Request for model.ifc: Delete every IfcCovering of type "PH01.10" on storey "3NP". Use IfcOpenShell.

First a look at what the model holds.

```python
import ifcopenshell
import ifcopenshell.util.element

model = ifcopenshell.open("model.ifc")
print(model.schema)
storey = next(s for s in model.by_type("IfcBuildingStorey") if s.Name == "3NP")
coverings = [e for e in ifcopenshell.util.element.get_decomposition(storey) if e.is_a("IfcCovering")]
seen = {}
for e in coverings:
    element_type = ifcopenshell.util.element.get_type(e)
    name = element_type.Name if element_type not in (None, e) else None
    seen[name] = seen.get(name, 0) + 1
for name, count in sorted(seen.items(), key=str):
    print(count, "x", name)
```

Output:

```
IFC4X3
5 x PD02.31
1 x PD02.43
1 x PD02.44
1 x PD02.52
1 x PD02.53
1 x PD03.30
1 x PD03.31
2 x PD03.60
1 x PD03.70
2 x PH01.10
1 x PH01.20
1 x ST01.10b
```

```python
import ifcopenshell
import ifcopenshell.api.root
import ifcopenshell.util.element

model = ifcopenshell.open("model.ifc")

storey = next(s for s in model.by_type("IfcBuildingStorey") if s.Name == "3NP")
coverings = [e for e in ifcopenshell.util.element.get_decomposition(storey) if e.is_a("IfcCovering")]
targets = [e for e in coverings if (t := ifcopenshell.util.element.get_type(e)) not in (None, e) and t.Name == "PH01.10"]

for e in targets:
    ifcopenshell.api.root.remove_product(model, product=e)
print(len(targets), "removed")

model.write("model_rev.ifc")
```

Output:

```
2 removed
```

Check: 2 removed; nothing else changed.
